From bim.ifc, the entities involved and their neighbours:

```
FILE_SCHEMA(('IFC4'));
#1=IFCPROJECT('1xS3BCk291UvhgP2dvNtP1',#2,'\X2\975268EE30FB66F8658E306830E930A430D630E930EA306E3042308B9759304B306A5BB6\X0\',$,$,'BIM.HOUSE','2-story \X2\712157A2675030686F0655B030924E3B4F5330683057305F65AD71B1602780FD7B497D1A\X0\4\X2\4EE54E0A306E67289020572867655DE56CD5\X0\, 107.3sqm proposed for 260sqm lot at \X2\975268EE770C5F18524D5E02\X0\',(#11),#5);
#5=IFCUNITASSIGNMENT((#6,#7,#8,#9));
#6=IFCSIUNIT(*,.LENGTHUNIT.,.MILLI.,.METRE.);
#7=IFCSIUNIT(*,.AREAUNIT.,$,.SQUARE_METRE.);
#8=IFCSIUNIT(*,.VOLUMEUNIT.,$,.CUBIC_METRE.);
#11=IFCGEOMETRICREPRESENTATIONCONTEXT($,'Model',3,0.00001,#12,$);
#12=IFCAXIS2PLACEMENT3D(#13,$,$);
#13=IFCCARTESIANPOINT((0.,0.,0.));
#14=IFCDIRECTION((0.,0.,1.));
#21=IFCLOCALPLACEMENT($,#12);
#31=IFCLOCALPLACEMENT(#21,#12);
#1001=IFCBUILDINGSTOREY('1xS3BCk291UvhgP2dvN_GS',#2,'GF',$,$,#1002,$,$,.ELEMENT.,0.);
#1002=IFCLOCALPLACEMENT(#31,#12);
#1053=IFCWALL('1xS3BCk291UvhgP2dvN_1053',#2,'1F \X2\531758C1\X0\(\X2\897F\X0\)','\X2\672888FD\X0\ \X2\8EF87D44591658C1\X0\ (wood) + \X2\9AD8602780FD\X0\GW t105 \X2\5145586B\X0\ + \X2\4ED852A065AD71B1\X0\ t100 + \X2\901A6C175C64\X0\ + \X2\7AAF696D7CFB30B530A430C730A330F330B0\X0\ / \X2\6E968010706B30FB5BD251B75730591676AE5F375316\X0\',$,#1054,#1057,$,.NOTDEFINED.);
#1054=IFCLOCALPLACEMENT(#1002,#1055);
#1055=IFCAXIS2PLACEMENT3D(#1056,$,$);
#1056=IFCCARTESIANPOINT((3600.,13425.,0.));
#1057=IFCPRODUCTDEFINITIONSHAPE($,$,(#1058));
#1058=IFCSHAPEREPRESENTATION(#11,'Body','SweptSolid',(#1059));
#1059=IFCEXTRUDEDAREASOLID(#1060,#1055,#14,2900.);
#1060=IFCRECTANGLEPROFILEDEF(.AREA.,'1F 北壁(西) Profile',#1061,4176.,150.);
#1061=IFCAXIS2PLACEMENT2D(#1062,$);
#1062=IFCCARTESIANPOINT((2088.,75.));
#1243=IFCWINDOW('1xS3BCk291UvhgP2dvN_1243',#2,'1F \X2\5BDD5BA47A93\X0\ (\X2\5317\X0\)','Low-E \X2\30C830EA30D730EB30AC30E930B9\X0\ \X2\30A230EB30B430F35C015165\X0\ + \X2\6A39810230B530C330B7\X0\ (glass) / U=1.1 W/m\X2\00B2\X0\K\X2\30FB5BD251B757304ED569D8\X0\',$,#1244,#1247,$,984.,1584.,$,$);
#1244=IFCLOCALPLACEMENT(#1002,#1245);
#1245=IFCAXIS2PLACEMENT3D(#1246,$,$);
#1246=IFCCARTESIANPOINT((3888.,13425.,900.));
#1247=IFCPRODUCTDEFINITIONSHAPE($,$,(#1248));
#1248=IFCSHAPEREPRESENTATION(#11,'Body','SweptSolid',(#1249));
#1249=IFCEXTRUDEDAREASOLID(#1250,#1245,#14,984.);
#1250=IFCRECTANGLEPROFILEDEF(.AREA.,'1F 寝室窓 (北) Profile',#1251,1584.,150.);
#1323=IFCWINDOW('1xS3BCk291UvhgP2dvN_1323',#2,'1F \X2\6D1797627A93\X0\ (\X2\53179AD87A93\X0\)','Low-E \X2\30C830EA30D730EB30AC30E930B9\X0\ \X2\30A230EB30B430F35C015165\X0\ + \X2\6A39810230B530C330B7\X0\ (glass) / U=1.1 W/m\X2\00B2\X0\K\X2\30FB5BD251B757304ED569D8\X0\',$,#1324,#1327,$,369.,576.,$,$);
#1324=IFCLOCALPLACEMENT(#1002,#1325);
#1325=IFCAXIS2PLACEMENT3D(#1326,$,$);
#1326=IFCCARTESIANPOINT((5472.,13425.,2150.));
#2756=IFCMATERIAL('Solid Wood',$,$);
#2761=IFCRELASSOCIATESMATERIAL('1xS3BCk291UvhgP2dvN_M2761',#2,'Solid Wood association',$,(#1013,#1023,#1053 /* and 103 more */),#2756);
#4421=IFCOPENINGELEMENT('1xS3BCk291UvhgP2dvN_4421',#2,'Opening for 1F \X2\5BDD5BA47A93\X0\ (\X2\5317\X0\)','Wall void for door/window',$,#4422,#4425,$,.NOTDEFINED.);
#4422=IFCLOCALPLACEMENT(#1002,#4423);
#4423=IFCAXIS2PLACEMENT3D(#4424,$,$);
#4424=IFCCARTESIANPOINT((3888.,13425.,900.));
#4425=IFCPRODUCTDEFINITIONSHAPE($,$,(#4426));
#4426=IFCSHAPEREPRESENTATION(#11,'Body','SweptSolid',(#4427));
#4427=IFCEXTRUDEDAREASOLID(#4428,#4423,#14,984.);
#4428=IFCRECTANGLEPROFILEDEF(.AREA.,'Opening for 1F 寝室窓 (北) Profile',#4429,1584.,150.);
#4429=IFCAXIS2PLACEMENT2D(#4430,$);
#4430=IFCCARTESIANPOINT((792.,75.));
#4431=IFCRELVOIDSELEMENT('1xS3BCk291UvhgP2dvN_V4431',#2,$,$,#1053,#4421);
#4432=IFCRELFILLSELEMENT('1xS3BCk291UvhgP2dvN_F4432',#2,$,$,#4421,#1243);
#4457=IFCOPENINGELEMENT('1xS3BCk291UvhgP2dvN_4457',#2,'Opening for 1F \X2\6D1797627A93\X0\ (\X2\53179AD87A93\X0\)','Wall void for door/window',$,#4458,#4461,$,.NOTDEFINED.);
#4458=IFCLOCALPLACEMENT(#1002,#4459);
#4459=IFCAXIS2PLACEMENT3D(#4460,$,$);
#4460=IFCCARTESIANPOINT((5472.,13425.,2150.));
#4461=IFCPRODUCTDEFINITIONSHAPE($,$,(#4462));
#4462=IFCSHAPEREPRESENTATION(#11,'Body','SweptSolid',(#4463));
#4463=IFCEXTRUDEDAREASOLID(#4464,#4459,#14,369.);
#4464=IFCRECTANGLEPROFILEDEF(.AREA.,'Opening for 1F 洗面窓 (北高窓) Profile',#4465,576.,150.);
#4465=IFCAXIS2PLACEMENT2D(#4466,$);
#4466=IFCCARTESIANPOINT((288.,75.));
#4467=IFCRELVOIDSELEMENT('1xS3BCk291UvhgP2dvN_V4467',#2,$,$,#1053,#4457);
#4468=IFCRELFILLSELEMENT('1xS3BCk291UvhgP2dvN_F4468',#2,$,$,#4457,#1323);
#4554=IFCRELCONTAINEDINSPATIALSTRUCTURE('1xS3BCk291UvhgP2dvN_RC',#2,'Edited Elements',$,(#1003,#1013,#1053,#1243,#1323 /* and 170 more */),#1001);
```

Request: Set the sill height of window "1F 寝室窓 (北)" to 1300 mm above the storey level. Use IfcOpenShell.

```python
import numpy as np
import ifcopenshell
import ifcopenshell.api.geometry
import ifcopenshell.geom
import ifcopenshell.util.element
import ifcopenshell.util.placement
import ifcopenshell.util.shape
import ifcopenshell.util.unit

model = ifcopenshell.open("bim.ifc")
unit_scale = ifcopenshell.util.unit.calculate_unit_scale(model)

window = model.by_guid("1xS3BCk291UvhgP2dvN_1243")
opening = window.FillsVoids[0].RelatingOpeningElement
storey = ifcopenshell.util.element.get_container(window, ifc_class="IfcBuildingStorey")
level = ifcopenshell.util.placement.get_local_placement(storey.ObjectPlacement)[2, 3]

# The opening's origin need not be at the sill, so measure its lowest point.
shape = ifcopenshell.geom.create_shape(ifcopenshell.geom.settings(), opening)
bottom = ifcopenshell.util.shape.get_shape_bottom_elevation(shape, shape.geometry) / unit_scale
dz = level + 1300.0 - bottom

shift = np.array([0.0, 0.0, dz])
# The window is not placed relative to its opening, so move both.
for product in (opening, window):
    matrix = ifcopenshell.util.placement.get_local_placement(product.ObjectPlacement)
    matrix[:3, 3] += shift
    ifcopenshell.api.geometry.edit_object_placement(model, product=product, matrix=matrix, is_si=False)

print(f"moved by {dz * unit_scale:+.3f} m")

model.write("bim_rev.ifc")
```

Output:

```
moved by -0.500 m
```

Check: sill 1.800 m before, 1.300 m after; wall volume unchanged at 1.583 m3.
